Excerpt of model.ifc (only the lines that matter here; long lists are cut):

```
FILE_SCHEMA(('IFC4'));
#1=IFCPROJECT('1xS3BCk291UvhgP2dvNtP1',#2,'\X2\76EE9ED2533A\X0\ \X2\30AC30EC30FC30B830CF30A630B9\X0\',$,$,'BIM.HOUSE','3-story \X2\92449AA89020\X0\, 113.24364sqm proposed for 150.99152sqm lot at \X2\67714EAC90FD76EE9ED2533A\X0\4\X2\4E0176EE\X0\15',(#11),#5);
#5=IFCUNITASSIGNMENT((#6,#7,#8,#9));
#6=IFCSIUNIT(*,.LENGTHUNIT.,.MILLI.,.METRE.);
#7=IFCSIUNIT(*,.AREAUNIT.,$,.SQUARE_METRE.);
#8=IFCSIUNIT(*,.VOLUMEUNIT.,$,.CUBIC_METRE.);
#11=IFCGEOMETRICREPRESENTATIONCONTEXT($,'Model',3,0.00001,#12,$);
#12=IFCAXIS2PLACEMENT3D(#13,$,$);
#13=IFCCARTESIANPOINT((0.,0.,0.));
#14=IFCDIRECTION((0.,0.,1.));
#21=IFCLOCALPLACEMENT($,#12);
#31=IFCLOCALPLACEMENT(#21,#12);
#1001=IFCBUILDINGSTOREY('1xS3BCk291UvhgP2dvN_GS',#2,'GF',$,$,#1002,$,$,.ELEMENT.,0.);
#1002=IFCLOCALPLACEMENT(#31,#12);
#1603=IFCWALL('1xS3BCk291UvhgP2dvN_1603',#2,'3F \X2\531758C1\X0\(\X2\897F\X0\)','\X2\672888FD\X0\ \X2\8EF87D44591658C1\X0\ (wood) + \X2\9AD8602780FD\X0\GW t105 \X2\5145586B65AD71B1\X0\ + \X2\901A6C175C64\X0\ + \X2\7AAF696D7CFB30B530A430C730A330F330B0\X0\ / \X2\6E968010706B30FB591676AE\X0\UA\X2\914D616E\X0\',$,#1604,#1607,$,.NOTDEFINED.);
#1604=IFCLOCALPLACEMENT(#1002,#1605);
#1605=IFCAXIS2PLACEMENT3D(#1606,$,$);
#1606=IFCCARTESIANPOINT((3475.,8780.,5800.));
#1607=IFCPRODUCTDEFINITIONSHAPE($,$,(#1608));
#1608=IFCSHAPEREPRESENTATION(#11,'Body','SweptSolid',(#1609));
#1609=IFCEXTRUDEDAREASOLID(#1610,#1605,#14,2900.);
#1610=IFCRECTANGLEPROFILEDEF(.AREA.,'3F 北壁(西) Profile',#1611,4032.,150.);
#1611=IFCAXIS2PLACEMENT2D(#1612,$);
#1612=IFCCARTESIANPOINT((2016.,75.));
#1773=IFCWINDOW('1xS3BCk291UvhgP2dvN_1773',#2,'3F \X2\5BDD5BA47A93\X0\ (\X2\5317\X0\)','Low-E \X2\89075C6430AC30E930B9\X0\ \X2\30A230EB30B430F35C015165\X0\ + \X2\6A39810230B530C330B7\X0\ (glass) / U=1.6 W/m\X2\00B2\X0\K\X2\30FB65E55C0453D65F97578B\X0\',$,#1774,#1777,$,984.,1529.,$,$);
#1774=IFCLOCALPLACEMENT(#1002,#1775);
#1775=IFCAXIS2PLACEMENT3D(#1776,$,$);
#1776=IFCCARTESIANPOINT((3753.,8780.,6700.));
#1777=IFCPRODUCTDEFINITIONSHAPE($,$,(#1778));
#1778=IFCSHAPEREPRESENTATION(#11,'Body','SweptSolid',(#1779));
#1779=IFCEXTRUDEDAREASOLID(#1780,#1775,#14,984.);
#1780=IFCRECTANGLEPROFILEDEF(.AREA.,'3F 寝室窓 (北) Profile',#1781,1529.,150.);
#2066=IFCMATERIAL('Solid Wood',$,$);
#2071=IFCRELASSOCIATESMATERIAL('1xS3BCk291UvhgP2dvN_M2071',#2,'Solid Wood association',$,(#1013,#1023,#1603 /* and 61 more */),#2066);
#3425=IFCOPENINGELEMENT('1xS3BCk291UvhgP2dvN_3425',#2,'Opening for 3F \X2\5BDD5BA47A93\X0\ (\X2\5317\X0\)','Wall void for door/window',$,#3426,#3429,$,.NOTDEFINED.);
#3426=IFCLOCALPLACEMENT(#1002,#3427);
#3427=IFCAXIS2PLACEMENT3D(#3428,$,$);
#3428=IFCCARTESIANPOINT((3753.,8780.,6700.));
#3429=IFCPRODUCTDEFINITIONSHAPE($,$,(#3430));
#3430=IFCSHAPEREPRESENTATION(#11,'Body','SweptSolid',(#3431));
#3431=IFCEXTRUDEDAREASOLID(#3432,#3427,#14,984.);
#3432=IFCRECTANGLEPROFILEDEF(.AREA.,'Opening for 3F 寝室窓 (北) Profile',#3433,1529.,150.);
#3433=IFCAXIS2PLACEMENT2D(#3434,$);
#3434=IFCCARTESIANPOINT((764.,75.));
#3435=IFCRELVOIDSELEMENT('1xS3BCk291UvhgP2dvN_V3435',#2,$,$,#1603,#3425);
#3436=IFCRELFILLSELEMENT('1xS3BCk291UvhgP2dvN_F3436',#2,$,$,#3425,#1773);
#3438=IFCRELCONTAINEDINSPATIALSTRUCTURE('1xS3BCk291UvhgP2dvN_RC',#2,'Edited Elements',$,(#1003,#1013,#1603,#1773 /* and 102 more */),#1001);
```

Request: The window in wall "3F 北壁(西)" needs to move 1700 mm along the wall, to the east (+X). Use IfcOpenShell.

```python
import ifcopenshell
import ifcopenshell.api.geometry
import ifcopenshell.util.placement

model = ifcopenshell.open("model.ifc")

window = model.by_guid("1xS3BCk291UvhgP2dvN_1773")
opening = window.FillsVoids[0].RelatingOpeningElement
wall = opening.VoidsElements[0].RelatingBuildingElement

wall_matrix = ifcopenshell.util.placement.get_local_placement(wall.ObjectPlacement)
shift = wall_matrix[:3, 0] * 1700.0
before = ifcopenshell.util.placement.get_local_placement(window.ObjectPlacement)[:3, 3].copy()

# The window is not placed relative to its opening, so move both.
for product in (opening, window):
    matrix = ifcopenshell.util.placement.get_local_placement(product.ObjectPlacement)
    matrix[:3, 3] += shift
    ifcopenshell.api.geometry.edit_object_placement(model, product=product, matrix=matrix, is_si=False)

after = ifcopenshell.util.placement.get_local_placement(window.ObjectPlacement)[:3, 3]
print("window moved by", (after - before).round(3) + 0.0)

model.write("model-out.ifc")
```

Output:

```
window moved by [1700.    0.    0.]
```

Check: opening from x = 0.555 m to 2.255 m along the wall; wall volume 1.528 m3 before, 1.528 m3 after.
